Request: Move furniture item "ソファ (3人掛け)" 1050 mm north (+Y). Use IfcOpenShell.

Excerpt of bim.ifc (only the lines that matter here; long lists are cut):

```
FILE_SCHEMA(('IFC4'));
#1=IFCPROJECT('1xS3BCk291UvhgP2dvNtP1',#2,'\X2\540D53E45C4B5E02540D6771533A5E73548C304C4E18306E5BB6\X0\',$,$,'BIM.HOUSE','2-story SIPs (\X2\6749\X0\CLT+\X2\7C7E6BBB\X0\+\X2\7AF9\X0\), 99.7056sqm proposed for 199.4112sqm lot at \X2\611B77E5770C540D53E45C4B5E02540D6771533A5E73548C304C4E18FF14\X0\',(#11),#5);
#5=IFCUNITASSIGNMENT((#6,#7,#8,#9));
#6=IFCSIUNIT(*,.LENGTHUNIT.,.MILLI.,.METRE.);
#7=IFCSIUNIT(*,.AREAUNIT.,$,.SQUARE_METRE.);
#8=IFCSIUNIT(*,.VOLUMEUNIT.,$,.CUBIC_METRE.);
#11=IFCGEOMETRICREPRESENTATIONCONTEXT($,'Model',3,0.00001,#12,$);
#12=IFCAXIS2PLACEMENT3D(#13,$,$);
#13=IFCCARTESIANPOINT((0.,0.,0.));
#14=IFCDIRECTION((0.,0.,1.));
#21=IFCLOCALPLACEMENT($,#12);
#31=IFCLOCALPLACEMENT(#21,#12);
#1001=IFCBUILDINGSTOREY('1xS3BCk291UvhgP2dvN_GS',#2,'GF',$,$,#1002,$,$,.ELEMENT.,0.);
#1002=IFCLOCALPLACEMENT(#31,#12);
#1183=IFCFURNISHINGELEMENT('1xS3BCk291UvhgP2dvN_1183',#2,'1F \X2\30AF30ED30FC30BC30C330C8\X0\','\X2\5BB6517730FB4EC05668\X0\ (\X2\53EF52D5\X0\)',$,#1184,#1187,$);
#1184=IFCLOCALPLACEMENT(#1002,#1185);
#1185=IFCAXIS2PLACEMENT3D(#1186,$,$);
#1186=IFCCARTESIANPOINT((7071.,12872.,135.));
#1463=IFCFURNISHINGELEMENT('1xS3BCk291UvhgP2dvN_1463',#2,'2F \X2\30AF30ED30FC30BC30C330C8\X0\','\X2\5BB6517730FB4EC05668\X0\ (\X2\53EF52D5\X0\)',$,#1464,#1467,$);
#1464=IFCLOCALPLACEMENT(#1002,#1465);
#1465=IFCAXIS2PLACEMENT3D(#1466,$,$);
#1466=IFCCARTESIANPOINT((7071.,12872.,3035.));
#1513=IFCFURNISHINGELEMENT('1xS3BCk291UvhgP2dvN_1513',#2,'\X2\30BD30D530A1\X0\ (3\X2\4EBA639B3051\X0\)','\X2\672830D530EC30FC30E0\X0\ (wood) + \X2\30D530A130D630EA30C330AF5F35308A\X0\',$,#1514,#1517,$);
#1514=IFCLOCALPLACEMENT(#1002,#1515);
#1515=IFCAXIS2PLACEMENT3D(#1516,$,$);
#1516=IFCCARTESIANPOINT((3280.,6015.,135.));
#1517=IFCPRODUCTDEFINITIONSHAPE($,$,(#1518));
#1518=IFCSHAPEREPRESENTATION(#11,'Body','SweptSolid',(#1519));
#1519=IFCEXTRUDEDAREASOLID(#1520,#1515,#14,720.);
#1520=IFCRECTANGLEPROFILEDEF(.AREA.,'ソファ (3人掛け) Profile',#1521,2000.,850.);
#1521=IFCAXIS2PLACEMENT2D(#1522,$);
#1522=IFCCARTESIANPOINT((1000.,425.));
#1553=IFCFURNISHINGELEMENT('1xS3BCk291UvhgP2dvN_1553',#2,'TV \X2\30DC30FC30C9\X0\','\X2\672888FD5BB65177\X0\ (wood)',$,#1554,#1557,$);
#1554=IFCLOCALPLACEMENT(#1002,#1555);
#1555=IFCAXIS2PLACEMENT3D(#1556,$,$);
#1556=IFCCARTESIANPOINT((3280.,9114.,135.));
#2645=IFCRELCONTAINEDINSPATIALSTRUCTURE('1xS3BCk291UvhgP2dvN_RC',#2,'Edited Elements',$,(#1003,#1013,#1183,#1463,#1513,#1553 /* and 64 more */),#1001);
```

```python
import ifcopenshell
import ifcopenshell.api.geometry
import ifcopenshell.util.placement
import ifcopenshell.util.unit

model = ifcopenshell.open("bim.ifc")
unit_scale = ifcopenshell.util.unit.calculate_unit_scale(model)

item = model.by_id(1513)
matrix = ifcopenshell.util.placement.get_local_placement(item.ObjectPlacement)
matrix[1, 3] += 1.05 / unit_scale
ifcopenshell.api.geometry.edit_object_placement(model, product=item, matrix=matrix, is_si=False)

print(ifcopenshell.util.placement.get_local_placement(item.ObjectPlacement).round(3) + 0.0)

model.write("bim_rev.ifc")
```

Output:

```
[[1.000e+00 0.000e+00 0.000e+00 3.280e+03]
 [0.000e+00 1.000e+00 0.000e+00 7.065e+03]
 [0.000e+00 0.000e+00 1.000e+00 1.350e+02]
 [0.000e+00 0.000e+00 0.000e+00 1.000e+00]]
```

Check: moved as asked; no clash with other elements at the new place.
